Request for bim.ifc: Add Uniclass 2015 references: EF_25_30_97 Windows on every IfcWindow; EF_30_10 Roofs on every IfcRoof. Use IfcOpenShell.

First a look at what the model holds.

```python
import ifcopenshell

model = ifcopenshell.open("bim.ifc")
print(model.schema)
print("classifications:", [c.Name for c in model.by_type("IfcClassification")])
for ifc_class in ("IfcDoor", "IfcRoof", "IfcStair", "IfcWall", "IfcWindow"):
    print(ifc_class, len(model.by_type(ifc_class)))
```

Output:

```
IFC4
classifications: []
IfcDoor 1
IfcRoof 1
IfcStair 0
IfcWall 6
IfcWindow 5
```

```python
import ifcopenshell
import ifcopenshell.api.classification

model = ifcopenshell.open("bim.ifc")

system = ifcopenshell.api.classification.add_classification(model, classification="Uniclass 2015")

codes = {
    "IfcWindow": ("EF_25_30_97", "Windows"),
    "IfcRoof": ("EF_30_10", "Roofs"),
}
for ifc_class, (code, name) in codes.items():
    products = model.by_type(ifc_class)
    ifcopenshell.api.classification.add_reference(
        model, products=products, classification=system, identification=code, name=name
    )
    print(code, len(products))

model.write("bim_v2.ifc")
```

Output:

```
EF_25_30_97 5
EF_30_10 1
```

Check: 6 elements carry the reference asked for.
